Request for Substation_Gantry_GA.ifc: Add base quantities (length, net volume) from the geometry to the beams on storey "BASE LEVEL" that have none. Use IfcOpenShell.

First a look at what the model holds.

```python
import ifcopenshell
import ifcopenshell.util.element
import ifcopenshell.util.unit

model = ifcopenshell.open("Substation_Gantry_GA.ifc")
print(model.schema)
for unit_type in ("LENGTHUNIT", "AREAUNIT", "VOLUMEUNIT"):
    print(unit_type, ifcopenshell.util.unit.calculate_unit_scale(model, unit_type))
storey = next(s for s in model.by_type("IfcBuildingStorey") if s.Name == "BASE LEVEL")
beams = [e for e in ifcopenshell.util.element.get_decomposition(storey) if e.is_a("IfcBeam")]
for e in sorted(beams, key=lambda e: e.id()):
    print(e.id(), e.is_a(), e.Name, list(ifcopenshell.util.element.get_psets(e, qtos_only=True)), sep=" | ")
```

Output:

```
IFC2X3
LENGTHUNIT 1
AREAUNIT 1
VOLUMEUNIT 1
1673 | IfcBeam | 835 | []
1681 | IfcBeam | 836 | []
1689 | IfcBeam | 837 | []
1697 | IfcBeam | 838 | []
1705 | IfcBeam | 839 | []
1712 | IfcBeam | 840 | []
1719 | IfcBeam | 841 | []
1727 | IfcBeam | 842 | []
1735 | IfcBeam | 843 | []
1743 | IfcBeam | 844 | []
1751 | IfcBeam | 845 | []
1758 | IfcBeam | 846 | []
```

```python
import ifcopenshell
import ifcopenshell.api.pset
import ifcopenshell.geom
import ifcopenshell.util.element
import ifcopenshell.util.shape
import ifcopenshell.util.unit

model = ifcopenshell.open("Substation_Gantry_GA.ifc")
unit_scale = ifcopenshell.util.unit.calculate_unit_scale(model)
volume_scale = ifcopenshell.util.unit.calculate_unit_scale(model, "VOLUMEUNIT")
settings = ifcopenshell.geom.settings()

storey = next(s for s in model.by_type("IfcBuildingStorey") if s.Name == "BASE LEVEL")
beams = [e for e in ifcopenshell.util.element.get_decomposition(storey) if e.is_a("IfcBeam")]

for e in sorted(beams, key=lambda e: e.id()):
    if ifcopenshell.util.element.get_psets(e, qtos_only=True, should_inherit=False):
        continue
    # Geometry comes back in metres, in the element's own axes.
    shape = ifcopenshell.geom.create_shape(settings, e)
    values = {
        "Length": ifcopenshell.util.shape.get_max_xyz(shape.geometry) / unit_scale,
        "NetVolume": ifcopenshell.util.shape.get_volume(shape.geometry) / volume_scale,
    }
    qto = ifcopenshell.api.pset.add_qto(model, product=e, name="BaseQuantities")
    ifcopenshell.api.pset.edit_qto(model, qto=qto, properties=values)
    print(e.id(), {k: round(v, 3) for k, v in values.items()})

model.write("Substation_Gantry_GA-out.ifc")
```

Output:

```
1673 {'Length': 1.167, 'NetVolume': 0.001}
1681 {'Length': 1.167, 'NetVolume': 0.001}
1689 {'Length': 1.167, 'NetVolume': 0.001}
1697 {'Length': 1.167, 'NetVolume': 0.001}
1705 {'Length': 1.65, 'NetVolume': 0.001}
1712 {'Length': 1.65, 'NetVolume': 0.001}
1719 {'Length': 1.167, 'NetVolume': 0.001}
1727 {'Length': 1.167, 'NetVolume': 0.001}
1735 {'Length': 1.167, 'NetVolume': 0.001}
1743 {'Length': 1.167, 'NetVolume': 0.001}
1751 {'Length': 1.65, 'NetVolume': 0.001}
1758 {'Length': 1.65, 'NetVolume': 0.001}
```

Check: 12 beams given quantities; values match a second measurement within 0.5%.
